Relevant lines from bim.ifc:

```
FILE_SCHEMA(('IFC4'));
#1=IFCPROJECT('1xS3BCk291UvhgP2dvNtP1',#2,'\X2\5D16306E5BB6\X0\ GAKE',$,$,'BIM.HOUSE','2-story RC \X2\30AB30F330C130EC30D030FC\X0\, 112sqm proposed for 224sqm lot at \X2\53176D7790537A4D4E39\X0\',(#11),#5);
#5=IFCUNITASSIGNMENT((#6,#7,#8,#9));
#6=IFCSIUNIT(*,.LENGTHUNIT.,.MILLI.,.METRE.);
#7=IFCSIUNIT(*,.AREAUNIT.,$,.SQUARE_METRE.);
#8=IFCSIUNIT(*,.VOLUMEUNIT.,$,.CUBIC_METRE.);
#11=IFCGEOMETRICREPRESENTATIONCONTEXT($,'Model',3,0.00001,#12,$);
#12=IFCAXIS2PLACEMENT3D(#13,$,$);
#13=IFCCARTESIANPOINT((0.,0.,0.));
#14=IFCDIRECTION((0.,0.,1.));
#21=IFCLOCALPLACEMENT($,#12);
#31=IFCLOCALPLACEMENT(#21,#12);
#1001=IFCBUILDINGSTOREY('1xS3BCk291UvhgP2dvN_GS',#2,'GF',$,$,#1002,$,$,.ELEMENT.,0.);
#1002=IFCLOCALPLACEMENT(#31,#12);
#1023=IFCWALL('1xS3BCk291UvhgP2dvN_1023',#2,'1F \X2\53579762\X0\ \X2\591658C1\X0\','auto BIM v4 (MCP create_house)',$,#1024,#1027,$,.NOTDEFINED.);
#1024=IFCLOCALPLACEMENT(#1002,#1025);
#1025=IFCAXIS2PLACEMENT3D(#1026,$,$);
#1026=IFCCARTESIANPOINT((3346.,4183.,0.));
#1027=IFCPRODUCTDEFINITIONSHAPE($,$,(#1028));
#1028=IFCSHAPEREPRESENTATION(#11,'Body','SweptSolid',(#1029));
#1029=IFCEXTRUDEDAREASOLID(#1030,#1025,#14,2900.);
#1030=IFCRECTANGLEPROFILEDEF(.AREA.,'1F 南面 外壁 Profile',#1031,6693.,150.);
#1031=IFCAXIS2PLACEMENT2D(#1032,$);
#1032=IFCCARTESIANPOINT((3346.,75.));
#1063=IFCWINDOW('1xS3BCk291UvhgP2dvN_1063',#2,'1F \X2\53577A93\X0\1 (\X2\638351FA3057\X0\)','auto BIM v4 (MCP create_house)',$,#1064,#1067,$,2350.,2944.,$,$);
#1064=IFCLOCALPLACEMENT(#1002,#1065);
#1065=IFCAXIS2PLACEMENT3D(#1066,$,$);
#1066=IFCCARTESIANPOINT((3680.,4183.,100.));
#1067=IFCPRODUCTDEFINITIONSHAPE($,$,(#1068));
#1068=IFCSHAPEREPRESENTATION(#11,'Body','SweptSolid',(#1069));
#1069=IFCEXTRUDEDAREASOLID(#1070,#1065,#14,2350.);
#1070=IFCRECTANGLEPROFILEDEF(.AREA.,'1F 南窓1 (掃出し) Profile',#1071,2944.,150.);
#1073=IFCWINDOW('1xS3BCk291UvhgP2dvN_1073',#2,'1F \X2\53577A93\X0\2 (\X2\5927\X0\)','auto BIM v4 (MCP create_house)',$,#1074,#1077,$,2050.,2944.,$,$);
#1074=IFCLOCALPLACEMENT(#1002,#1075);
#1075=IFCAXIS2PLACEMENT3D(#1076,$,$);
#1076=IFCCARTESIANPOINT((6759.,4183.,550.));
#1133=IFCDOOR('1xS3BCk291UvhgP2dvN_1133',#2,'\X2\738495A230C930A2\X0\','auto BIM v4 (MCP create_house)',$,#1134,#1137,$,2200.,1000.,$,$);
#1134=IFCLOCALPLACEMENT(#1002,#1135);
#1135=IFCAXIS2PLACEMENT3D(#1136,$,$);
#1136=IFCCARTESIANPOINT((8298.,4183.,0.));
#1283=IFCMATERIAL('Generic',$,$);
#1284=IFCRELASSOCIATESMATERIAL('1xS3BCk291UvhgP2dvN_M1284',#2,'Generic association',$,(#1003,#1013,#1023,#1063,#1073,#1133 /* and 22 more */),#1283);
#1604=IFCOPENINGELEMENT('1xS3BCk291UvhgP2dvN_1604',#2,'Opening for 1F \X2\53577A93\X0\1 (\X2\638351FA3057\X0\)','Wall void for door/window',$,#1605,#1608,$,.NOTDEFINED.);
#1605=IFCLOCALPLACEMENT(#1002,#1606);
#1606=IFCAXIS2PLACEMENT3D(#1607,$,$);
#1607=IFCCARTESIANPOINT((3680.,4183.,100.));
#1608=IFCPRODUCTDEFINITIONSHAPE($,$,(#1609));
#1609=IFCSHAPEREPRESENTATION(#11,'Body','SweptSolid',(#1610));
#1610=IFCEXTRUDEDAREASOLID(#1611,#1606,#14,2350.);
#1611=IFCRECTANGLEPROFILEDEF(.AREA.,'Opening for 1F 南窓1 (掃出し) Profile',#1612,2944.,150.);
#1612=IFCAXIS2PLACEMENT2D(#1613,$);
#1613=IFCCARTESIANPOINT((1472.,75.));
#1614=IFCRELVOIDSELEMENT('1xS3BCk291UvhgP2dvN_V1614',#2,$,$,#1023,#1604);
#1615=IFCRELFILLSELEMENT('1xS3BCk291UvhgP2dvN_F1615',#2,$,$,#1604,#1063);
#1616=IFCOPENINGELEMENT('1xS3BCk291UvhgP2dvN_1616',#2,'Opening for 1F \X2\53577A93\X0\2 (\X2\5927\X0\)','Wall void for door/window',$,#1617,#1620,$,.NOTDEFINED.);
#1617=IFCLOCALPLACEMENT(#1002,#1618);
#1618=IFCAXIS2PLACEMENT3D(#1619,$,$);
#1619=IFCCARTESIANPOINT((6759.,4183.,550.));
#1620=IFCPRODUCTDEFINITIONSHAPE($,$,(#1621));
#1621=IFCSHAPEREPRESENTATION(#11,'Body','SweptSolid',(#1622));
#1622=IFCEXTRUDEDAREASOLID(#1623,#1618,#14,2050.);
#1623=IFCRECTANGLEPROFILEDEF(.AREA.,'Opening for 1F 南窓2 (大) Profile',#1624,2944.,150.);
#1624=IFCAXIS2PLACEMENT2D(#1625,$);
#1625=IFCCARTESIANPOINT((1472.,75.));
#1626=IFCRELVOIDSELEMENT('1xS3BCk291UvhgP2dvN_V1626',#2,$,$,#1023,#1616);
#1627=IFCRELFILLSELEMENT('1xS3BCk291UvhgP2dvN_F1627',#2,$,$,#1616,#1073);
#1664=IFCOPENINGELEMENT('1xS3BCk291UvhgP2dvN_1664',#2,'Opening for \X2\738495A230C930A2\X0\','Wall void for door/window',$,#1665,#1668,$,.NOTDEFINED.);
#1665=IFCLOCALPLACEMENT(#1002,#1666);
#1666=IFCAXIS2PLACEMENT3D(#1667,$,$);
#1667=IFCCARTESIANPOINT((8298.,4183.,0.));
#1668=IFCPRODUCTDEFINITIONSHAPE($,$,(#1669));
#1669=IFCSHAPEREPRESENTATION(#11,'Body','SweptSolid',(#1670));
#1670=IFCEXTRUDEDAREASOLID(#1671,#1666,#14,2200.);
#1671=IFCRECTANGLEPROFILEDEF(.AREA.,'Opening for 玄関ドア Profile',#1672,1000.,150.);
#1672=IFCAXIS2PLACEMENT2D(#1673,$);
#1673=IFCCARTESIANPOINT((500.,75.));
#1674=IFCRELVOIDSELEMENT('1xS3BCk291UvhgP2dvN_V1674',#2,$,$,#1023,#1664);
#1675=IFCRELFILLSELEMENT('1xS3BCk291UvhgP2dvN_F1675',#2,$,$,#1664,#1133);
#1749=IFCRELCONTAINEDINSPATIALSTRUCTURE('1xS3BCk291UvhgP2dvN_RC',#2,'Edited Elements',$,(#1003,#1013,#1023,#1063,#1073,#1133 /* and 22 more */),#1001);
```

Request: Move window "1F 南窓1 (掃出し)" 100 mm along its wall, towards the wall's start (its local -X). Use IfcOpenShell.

```python
import ifcopenshell
import ifcopenshell.api.geometry
import ifcopenshell.util.placement
import ifcopenshell.util.unit

model = ifcopenshell.open("bim.ifc")
unit_scale = ifcopenshell.util.unit.calculate_unit_scale(model)

window = model.by_guid("1xS3BCk291UvhgP2dvN_1063")
opening = window.FillsVoids[0].RelatingOpeningElement
wall = opening.VoidsElements[0].RelatingBuildingElement

wall_matrix = ifcopenshell.util.placement.get_local_placement(wall.ObjectPlacement)
shift = wall_matrix[:3, 0] * -0.1 / unit_scale
before = ifcopenshell.util.placement.get_local_placement(window.ObjectPlacement)[:3, 3].copy()

# The window is not placed relative to its opening, so move both.
for product in (opening, window):
    matrix = ifcopenshell.util.placement.get_local_placement(product.ObjectPlacement)
    matrix[:3, 3] += shift
    ifcopenshell.api.geometry.edit_object_placement(model, product=product, matrix=matrix, is_si=False)

after = ifcopenshell.util.placement.get_local_placement(window.ObjectPlacement)[:3, 3]
print("window moved by", (after - before).round(3) + 0.0)

model.write("bim_edited.ifc")
```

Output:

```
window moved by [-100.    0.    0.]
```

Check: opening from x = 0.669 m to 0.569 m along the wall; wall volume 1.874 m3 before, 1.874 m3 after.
